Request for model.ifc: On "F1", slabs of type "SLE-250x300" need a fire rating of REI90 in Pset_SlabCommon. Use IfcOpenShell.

First a look at what the model holds.

```python
import ifcopenshell
import ifcopenshell.util.element

model = ifcopenshell.open("model.ifc")
print(model.schema)
storey = next(s for s in model.by_type("IfcBuildingStorey") if s.Name == "F1")
slabs = [e for e in ifcopenshell.util.element.get_decomposition(storey) if e.is_a("IfcSlab")]
seen = {}
for e in slabs:
    element_type = ifcopenshell.util.element.get_type(e)
    key = (element_type.Name if element_type != e and element_type else None, ifcopenshell.util.element.get_pset(e, "Pset_SlabCommon", "FireRating"))
    seen[key] = seen.get(key, 0) + 1
for (name, value), count in sorted(seen.items(), key=str):
    print(count, "x", name, "|", value)
```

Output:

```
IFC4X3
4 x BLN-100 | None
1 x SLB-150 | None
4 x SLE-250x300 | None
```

```python
import ifcopenshell
import ifcopenshell.api.pset
import ifcopenshell.util.element

model = ifcopenshell.open("model.ifc")

storey = next(s for s in model.by_type("IfcBuildingStorey") if s.Name == "F1")
slabs = [e for e in ifcopenshell.util.element.get_decomposition(storey) if e.is_a("IfcSlab")]

count = 0
for e in slabs:
    element_type = ifcopenshell.util.element.get_type(e)
    if element_type in (None, e) or element_type.Name != "SLE-250x300":
        continue
    # add_pset returns the element's existing set when there is one.
    pset = ifcopenshell.api.pset.add_pset(model, product=e, name="Pset_SlabCommon")
    ifcopenshell.api.pset.edit_pset(model, pset=pset, properties={"FireRating": "REI90"})
    count += 1

print(count, "slabs updated")

model.write("model_v2.ifc")
```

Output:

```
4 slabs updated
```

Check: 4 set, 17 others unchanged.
